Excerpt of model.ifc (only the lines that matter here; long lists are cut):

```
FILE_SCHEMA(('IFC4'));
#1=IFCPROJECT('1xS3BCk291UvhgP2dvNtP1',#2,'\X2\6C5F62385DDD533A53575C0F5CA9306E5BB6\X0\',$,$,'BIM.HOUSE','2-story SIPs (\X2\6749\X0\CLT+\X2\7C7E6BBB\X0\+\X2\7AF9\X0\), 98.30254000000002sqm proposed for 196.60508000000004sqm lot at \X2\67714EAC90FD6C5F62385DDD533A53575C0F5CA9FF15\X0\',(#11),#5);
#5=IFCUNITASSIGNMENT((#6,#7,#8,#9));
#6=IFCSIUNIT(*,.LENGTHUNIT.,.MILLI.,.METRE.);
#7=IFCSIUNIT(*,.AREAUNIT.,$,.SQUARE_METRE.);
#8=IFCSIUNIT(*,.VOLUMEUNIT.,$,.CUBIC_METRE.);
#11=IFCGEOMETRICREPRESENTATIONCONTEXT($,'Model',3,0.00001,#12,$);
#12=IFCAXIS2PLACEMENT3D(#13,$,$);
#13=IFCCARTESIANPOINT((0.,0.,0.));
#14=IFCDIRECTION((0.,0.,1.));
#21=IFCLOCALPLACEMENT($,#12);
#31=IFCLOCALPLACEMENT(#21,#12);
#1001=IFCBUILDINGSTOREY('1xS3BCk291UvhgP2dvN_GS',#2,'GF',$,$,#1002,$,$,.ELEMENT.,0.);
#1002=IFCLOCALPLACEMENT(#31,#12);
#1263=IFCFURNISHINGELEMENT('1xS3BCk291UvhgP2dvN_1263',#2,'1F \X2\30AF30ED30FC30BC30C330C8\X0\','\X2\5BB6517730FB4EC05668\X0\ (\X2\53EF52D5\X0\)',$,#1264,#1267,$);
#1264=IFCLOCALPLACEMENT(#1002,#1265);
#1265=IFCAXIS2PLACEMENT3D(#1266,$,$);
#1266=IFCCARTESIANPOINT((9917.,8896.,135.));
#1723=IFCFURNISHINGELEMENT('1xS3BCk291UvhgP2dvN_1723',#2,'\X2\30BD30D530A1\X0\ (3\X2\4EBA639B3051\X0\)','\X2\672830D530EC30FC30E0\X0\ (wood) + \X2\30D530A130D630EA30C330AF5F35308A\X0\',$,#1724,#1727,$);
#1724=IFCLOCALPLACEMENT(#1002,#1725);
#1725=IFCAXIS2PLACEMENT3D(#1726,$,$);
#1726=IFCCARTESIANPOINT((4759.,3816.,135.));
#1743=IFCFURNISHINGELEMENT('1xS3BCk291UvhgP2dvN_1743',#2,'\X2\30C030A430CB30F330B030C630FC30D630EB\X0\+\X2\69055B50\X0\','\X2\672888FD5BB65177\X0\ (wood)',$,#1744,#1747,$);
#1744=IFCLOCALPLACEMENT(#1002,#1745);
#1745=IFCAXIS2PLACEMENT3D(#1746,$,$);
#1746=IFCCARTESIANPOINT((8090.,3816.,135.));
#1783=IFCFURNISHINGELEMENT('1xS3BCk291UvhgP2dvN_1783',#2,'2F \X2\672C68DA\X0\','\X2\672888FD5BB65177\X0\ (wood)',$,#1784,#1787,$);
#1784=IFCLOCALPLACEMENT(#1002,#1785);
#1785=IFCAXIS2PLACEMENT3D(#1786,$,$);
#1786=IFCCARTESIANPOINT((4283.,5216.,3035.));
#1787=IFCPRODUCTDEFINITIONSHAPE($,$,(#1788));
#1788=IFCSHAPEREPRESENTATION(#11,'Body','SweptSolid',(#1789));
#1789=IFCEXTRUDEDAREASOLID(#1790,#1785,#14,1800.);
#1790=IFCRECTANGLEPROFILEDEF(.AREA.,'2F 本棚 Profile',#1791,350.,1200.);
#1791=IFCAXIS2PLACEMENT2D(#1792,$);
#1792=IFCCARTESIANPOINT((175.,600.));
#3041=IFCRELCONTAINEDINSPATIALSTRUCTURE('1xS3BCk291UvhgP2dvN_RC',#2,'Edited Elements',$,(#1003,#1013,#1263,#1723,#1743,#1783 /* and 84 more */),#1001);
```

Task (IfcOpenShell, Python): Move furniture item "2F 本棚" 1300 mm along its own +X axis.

```python
import ifcopenshell
import ifcopenshell.api.geometry
import ifcopenshell.util.placement
import ifcopenshell.util.unit

model = ifcopenshell.open("model.ifc")
unit_scale = ifcopenshell.util.unit.calculate_unit_scale(model)

item = model.by_id(1783)
matrix = ifcopenshell.util.placement.get_local_placement(item.ObjectPlacement)
matrix[:3, 3] += matrix[:3, 0] * 1.3 / unit_scale
ifcopenshell.api.geometry.edit_object_placement(model, product=item, matrix=matrix, is_si=False)

print(ifcopenshell.util.placement.get_local_placement(item.ObjectPlacement).round(3) + 0.0)

model.write("model_v2.ifc")
```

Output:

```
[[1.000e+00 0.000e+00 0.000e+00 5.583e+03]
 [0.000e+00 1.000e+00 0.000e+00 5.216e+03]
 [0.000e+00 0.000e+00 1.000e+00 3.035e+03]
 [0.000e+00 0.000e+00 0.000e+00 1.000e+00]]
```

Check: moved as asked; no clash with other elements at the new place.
